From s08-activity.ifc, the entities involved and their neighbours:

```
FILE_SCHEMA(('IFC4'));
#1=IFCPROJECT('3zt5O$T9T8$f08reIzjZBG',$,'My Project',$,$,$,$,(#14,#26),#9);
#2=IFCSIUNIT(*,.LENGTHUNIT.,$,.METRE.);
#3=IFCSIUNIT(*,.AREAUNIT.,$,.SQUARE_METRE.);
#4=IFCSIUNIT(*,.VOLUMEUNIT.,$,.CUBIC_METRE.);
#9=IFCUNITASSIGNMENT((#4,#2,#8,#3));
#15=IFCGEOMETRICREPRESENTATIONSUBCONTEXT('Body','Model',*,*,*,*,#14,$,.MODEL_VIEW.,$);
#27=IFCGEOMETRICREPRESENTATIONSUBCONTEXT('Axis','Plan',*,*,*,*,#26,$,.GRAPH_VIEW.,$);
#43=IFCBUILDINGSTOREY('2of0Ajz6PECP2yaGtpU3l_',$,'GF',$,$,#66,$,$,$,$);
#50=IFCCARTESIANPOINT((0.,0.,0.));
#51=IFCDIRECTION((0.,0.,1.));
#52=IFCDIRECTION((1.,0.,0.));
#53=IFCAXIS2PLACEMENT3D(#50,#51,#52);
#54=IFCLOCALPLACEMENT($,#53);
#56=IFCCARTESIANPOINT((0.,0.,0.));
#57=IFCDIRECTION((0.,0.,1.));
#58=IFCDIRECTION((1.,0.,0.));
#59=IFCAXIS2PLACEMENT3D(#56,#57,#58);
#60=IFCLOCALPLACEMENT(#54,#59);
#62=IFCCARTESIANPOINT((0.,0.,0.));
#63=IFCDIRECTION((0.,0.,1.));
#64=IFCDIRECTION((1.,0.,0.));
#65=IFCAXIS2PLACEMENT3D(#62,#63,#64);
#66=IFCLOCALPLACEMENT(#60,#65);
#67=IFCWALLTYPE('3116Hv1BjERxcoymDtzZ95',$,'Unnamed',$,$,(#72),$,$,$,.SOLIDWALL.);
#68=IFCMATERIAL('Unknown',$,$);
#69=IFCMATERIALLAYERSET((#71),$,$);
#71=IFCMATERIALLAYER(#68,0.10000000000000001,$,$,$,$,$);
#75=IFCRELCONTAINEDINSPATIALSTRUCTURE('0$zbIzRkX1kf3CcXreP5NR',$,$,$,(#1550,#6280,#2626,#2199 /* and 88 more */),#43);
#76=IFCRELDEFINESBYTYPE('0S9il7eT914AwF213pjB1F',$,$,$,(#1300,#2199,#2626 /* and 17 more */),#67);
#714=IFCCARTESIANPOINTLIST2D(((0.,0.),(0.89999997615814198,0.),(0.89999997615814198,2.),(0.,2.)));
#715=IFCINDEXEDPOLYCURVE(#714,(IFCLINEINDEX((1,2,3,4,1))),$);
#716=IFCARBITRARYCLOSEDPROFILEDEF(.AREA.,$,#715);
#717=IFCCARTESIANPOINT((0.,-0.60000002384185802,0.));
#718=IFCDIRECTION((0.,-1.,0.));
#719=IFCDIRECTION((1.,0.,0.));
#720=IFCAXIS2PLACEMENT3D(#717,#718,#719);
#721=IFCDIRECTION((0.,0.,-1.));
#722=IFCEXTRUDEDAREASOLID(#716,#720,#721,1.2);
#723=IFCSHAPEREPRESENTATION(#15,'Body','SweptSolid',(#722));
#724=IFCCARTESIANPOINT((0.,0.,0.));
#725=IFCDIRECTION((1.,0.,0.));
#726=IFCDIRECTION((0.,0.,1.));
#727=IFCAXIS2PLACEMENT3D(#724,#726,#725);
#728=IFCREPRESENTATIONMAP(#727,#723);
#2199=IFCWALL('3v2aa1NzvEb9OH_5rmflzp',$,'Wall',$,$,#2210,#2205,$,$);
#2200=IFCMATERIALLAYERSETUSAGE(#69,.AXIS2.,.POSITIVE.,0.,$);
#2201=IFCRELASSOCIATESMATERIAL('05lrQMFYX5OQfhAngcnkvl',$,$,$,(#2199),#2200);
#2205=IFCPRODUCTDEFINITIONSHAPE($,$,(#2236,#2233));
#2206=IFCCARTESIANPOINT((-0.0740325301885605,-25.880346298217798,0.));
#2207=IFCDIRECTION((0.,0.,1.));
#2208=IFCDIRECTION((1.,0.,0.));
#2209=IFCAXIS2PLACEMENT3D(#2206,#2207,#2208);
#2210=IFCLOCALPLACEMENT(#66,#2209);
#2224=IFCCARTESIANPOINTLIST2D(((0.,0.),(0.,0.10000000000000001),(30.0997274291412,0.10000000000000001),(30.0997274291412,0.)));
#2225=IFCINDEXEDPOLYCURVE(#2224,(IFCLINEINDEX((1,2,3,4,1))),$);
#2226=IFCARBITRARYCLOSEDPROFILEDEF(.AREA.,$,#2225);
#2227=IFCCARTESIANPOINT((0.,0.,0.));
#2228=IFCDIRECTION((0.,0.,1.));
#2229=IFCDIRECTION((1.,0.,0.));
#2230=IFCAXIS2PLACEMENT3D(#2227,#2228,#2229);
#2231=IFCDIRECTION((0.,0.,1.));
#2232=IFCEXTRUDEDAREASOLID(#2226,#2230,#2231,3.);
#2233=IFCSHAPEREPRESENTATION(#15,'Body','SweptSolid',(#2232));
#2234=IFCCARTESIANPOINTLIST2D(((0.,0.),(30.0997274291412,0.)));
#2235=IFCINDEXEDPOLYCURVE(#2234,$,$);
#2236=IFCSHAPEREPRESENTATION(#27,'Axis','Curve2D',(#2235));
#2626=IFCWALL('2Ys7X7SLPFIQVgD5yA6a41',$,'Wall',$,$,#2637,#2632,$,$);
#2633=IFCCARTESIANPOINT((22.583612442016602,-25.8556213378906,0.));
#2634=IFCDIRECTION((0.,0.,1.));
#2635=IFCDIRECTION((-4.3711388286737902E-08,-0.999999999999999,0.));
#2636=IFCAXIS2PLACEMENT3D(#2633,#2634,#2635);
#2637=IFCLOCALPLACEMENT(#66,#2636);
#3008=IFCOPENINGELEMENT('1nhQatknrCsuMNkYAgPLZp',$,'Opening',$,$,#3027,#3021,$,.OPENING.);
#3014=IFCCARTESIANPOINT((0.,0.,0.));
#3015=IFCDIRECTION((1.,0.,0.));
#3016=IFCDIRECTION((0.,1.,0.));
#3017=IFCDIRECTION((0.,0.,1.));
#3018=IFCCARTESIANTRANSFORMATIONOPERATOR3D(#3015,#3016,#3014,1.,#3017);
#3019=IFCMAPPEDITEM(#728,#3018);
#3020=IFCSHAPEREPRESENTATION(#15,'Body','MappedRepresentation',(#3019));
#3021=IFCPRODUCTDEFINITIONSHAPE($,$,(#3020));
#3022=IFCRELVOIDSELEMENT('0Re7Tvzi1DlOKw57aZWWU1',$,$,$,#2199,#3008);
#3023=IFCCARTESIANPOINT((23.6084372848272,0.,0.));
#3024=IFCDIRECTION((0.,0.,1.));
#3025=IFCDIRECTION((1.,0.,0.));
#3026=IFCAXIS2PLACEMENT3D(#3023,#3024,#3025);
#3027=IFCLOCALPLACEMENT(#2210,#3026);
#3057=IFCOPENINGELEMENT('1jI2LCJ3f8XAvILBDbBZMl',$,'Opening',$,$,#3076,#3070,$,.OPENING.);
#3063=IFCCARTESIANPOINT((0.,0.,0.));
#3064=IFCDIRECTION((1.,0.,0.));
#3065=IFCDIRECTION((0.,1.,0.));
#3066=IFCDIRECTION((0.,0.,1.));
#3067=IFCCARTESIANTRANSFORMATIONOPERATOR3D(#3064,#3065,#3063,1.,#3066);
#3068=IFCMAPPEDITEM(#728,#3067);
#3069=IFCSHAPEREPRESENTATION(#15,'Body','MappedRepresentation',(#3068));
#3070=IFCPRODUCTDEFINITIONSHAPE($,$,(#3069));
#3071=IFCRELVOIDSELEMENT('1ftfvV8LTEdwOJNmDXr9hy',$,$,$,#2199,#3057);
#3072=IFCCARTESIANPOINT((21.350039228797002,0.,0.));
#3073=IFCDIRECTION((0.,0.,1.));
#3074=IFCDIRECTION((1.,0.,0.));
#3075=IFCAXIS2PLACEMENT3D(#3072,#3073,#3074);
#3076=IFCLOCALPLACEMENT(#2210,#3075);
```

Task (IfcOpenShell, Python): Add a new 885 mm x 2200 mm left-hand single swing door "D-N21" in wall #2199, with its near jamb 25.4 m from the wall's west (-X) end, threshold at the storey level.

```python
import numpy as np
import ifcopenshell
import ifcopenshell.api.feature
import ifcopenshell.api.geometry
import ifcopenshell.api.root
import ifcopenshell.api.spatial
import ifcopenshell.geom
import ifcopenshell.util.element
import ifcopenshell.util.placement
import ifcopenshell.util.representation
import ifcopenshell.util.shape
import ifcopenshell.util.unit

model = ifcopenshell.open("s08-activity.ifc")
unit_scale = ifcopenshell.util.unit.calculate_unit_scale(model)
settings = ifcopenshell.geom.settings()


def volume(element):
    """Net volume in cubic metres, openings subtracted."""
    shape = ifcopenshell.geom.create_shape(settings, element)
    return ifcopenshell.util.shape.get_volume(shape.geometry)


wall = model.by_id(2199)
storey = ifcopenshell.util.element.get_container(wall, ifc_class="IfcBuildingStorey")
context = ifcopenshell.util.representation.get_context(model, "Model", "Body", "MODEL_VIEW")
before = volume(wall)

width, height, from_end, sill = 0.885, 2.2, 25.4, 0.0  # metres

# The wall runs along its own X axis, and the end named is its -X end.
wall_shape = ifcopenshell.geom.create_shape(settings, wall)
x, y, z = ifcopenshell.util.shape.get_vertices(wall_shape.geometry).T
start = x.min() + from_end
face, thickness = float(y.min()), float(y.max() - y.min())
wall_matrix = ifcopenshell.util.placement.get_local_placement(wall.ObjectPlacement)
level = ifcopenshell.util.placement.get_local_placement(storey.ObjectPlacement)[2, 3]


def in_wall(x, y):
    """Placement at x, y metres in the wall's axes, at sill height."""
    matrix = wall_matrix.copy()
    matrix[:, 3] = wall_matrix @ np.array([x / unit_scale, y / unit_scale, 0.0, 1.0])
    matrix[2, 3] = level + sill / unit_scale
    return matrix


# Opening: a box that overshoots both wall faces by 50 mm.
opening = ifcopenshell.api.root.create_entity(model, ifc_class="IfcOpeningElement", predefined_type="OPENING")
box = ifcopenshell.api.geometry.add_wall_representation(
    model, context=context, length=width, height=height, thickness=thickness + 0.1
)
ifcopenshell.api.geometry.assign_representation(model, product=opening, representation=box)
ifcopenshell.api.geometry.edit_object_placement(model, product=opening, matrix=in_wall(start, face - 0.05), is_si=False)
ifcopenshell.api.feature.add_feature(model, feature=opening, element=wall)

door = ifcopenshell.api.root.create_entity(model, ifc_class="IfcDoor", name="D-N21", predefined_type="DOOR")
door.OverallWidth, door.OverallHeight = width / unit_scale, height / unit_scale
door.OperationType = "SINGLE_SWING_LEFT"
body = ifcopenshell.api.geometry.add_door_representation(
    model,
    context=context,
    overall_width=door.OverallWidth,
    overall_height=door.OverallHeight,
    operation_type="SINGLE_SWING_LEFT",
    lining_properties={"LiningDepth": thickness / unit_scale, "ThresholdDepth": thickness / unit_scale},
)
ifcopenshell.api.geometry.assign_representation(model, product=door, representation=body)
ifcopenshell.api.spatial.assign_container(model, products=[door], relating_structure=storey)
ifcopenshell.api.feature.add_filling(model, opening=opening, element=door)

# The lining spans the wall, so the door starts at the wall face.
ifcopenshell.api.geometry.edit_object_placement(model, product=door, matrix=in_wall(start, face), is_si=False)

after = volume(wall)

print(f"wall volume {before:.3f} -> {after:.3f} m3")

model.write("s08-activity-out.ifc")
```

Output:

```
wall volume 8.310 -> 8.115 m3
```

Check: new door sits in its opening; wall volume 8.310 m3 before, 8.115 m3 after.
